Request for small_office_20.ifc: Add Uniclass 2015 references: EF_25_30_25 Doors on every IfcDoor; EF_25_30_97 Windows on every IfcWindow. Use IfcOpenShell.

First a look at what the model holds.

```python
import ifcopenshell

model = ifcopenshell.open("small_office_20.ifc")
print(model.schema)
print("classifications:", [c.Name for c in model.by_type("IfcClassification")])
for ifc_class in ("IfcDoor", "IfcRoof", "IfcStair", "IfcWall", "IfcWindow"):
    print(ifc_class, len(model.by_type(ifc_class)))
```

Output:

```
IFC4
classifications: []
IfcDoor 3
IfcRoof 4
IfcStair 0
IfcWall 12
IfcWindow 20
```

```python
import ifcopenshell
import ifcopenshell.api.classification

model = ifcopenshell.open("small_office_20.ifc")

system = ifcopenshell.api.classification.add_classification(model, classification="Uniclass 2015")

codes = {
    "IfcDoor": ("EF_25_30_25", "Doors"),
    "IfcWindow": ("EF_25_30_97", "Windows"),
}
for ifc_class, (code, name) in codes.items():
    products = model.by_type(ifc_class)
    ifcopenshell.api.classification.add_reference(
        model, products=products, classification=system, identification=code, name=name
    )
    print(code, len(products))

model.write("small_office_20-out.ifc")
```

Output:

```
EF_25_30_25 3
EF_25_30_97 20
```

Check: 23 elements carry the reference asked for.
